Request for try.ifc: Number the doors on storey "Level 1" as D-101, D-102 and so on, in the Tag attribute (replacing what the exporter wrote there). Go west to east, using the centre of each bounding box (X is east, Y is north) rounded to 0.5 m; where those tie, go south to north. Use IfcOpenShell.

First a look at what the model holds.

```python
import ifcopenshell
import ifcopenshell.util.element
import ifcopenshell.util.placement

model = ifcopenshell.open("try.ifc")
print(model.schema)
storey = next(s for s in model.by_type("IfcBuildingStorey") if s.Name == "Level 1")
doors = [e for e in ifcopenshell.util.element.get_decomposition(storey) if e.is_a("IfcDoor")]
for e in sorted(doors, key=lambda e: e.id()):
    origin = ifcopenshell.util.placement.get_local_placement(e.ObjectPlacement)[:3, 3]
    print(e.id(), e.Tag, e.Name, origin.round(2) + 0.0, sep=" | ")
```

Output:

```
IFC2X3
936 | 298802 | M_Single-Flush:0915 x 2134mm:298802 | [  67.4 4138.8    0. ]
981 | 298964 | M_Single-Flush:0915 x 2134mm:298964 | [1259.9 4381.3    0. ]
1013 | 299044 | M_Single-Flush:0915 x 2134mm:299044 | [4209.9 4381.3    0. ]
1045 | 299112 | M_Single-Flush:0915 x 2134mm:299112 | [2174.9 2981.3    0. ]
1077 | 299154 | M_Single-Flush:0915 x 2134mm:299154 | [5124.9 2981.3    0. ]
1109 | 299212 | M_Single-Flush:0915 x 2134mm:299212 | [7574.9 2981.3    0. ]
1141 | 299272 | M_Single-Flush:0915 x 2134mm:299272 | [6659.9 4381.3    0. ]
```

```python
import ifcopenshell
import ifcopenshell.geom
import ifcopenshell.util.element
import ifcopenshell.util.shape

model = ifcopenshell.open("try.ifc")
settings = ifcopenshell.geom.settings()
settings.set("use-world-coords", True)


def centre(element):
    shape = ifcopenshell.geom.create_shape(settings, element)
    return ifcopenshell.util.shape.get_bbox_centroid(shape.geometry)


storey = next(s for s in model.by_type("IfcBuildingStorey") if s.Name == "Level 1")
doors = [e for e in ifcopenshell.util.element.get_decomposition(storey) if e.is_a("IfcDoor")]

# Insertion points can sit at a corner or the storey origin, so sort by the geometry (in metres).
centres = {e: centre(e) for e in doors}
doors.sort(key=lambda e: (round(centres[e][0] / 0.5), centres[e][1]))

for i, e in enumerate(doors, start=1):
    number = f"D-1{i:02d}"
    e.Tag = number
    print(e.id(), number)

model.write("try_rev.ifc")
```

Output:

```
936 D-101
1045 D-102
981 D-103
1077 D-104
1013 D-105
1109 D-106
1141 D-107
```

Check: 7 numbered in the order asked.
